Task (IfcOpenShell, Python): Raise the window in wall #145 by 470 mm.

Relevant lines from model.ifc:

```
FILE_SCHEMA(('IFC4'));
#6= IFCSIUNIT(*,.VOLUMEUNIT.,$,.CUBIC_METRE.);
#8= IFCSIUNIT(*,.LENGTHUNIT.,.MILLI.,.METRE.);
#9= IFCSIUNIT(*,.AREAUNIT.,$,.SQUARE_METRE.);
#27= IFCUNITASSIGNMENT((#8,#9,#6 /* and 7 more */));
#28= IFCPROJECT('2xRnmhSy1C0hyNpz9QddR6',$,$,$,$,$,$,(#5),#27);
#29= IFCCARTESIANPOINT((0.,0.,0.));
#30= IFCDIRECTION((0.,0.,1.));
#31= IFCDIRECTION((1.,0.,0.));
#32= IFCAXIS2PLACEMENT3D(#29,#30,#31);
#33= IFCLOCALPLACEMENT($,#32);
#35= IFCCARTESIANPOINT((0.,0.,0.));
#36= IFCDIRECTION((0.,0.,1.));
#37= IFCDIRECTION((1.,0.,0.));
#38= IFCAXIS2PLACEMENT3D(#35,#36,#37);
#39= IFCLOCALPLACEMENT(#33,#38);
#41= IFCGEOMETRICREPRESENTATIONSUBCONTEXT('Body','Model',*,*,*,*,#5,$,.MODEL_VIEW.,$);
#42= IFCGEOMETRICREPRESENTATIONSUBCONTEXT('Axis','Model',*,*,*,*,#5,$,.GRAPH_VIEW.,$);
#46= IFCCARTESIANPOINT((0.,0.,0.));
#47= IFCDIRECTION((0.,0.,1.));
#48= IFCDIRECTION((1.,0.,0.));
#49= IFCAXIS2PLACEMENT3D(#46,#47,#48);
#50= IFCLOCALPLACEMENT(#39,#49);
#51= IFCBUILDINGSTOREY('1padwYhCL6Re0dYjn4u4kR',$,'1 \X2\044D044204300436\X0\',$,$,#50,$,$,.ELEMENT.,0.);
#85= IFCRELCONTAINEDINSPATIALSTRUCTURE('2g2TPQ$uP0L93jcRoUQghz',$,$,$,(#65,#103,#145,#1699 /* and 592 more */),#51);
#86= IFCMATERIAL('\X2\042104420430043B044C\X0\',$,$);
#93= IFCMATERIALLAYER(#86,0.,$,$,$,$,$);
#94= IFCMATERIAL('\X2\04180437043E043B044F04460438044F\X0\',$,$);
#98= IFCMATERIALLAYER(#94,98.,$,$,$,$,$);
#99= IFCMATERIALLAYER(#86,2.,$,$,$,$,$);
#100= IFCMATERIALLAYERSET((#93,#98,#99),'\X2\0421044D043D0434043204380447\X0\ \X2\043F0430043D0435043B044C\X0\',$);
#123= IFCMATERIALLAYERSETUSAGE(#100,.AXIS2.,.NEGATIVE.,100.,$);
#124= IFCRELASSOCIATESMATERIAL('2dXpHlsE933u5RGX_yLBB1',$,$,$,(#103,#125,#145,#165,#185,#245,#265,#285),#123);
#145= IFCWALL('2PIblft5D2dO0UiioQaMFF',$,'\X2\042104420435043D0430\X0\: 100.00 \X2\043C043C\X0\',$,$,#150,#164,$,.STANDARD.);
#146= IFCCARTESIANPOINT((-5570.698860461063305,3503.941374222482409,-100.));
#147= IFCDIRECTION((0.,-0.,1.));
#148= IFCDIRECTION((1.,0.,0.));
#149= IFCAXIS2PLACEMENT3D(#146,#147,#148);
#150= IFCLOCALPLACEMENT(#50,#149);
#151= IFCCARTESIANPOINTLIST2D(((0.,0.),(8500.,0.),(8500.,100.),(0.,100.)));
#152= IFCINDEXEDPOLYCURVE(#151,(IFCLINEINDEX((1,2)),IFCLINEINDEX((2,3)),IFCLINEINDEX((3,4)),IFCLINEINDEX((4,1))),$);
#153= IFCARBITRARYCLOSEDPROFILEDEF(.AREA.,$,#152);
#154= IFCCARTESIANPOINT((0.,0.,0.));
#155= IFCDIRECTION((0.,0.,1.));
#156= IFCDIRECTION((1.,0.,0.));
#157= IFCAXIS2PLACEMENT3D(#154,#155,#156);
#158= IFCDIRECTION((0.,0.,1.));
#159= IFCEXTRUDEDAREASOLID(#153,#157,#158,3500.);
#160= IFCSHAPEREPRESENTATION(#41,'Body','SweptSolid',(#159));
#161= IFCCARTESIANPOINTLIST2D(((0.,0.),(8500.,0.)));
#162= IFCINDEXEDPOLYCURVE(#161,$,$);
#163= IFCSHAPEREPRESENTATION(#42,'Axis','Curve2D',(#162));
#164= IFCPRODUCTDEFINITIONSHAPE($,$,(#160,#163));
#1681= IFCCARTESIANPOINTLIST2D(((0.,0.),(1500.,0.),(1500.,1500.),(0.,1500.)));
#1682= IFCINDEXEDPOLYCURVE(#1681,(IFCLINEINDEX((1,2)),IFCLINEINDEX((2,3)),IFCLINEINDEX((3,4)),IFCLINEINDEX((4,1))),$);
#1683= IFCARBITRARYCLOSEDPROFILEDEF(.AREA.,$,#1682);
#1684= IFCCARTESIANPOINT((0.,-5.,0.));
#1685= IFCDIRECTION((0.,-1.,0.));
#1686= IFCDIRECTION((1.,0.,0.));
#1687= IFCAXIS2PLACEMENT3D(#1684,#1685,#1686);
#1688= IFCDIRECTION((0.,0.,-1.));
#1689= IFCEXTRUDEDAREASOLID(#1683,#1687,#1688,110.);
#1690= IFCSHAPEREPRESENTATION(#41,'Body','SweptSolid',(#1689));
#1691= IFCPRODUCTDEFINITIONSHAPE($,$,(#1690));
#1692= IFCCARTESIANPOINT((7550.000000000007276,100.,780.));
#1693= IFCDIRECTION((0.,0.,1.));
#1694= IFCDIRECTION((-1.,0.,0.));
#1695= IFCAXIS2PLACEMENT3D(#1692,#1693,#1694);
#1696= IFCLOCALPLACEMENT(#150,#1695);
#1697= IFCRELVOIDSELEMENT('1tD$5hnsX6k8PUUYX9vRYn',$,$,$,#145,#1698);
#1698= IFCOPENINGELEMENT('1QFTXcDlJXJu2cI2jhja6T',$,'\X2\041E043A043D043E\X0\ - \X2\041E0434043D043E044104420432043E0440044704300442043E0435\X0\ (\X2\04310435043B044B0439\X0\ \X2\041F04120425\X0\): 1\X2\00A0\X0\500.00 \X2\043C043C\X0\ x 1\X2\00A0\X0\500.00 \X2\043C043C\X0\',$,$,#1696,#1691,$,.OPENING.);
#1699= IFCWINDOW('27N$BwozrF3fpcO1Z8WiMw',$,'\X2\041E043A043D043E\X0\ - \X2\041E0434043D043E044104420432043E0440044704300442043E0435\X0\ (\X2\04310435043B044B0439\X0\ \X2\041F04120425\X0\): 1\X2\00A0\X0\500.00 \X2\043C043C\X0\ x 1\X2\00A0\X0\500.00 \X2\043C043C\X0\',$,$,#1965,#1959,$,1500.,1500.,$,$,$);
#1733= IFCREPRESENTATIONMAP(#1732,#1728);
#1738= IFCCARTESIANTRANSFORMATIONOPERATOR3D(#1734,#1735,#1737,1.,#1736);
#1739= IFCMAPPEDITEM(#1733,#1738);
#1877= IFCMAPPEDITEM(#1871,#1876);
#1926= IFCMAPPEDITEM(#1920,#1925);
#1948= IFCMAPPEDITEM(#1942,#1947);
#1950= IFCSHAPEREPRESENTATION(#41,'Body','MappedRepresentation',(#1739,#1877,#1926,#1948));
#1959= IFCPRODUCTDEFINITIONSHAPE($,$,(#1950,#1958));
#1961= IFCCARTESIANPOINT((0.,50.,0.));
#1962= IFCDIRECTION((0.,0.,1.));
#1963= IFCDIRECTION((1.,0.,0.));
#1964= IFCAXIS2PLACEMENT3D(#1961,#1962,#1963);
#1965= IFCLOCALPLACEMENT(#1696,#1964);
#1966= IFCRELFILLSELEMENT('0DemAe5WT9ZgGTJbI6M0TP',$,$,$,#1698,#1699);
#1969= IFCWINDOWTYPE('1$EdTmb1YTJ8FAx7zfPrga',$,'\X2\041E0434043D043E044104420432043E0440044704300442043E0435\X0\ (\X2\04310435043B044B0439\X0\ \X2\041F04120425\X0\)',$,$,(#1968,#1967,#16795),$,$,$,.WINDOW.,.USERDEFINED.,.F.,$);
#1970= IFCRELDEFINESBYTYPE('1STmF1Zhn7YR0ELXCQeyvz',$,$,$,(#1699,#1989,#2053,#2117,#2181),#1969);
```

```python
import numpy as np
import ifcopenshell
import ifcopenshell.api.geometry
import ifcopenshell.util.placement
import ifcopenshell.util.unit

model = ifcopenshell.open("model.ifc")
unit_scale = ifcopenshell.util.unit.calculate_unit_scale(model)

window = model.by_guid("27N$BwozrF3fpcO1Z8WiMw")
opening = window.FillsVoids[0].RelatingOpeningElement
dz = 0.47 / unit_scale

shift = np.array([0.0, 0.0, dz])
# The window is placed relative to its opening, so it follows when the opening moves.
matrix = ifcopenshell.util.placement.get_local_placement(opening.ObjectPlacement)
matrix[:3, 3] += shift
ifcopenshell.api.geometry.edit_object_placement(
    model, product=opening, matrix=matrix, is_si=False, should_transform_children=True
)

print(f"moved by {dz * unit_scale:+.3f} m")

model.write("model_rev.ifc")
```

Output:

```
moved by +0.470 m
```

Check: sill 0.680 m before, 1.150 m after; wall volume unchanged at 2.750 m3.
